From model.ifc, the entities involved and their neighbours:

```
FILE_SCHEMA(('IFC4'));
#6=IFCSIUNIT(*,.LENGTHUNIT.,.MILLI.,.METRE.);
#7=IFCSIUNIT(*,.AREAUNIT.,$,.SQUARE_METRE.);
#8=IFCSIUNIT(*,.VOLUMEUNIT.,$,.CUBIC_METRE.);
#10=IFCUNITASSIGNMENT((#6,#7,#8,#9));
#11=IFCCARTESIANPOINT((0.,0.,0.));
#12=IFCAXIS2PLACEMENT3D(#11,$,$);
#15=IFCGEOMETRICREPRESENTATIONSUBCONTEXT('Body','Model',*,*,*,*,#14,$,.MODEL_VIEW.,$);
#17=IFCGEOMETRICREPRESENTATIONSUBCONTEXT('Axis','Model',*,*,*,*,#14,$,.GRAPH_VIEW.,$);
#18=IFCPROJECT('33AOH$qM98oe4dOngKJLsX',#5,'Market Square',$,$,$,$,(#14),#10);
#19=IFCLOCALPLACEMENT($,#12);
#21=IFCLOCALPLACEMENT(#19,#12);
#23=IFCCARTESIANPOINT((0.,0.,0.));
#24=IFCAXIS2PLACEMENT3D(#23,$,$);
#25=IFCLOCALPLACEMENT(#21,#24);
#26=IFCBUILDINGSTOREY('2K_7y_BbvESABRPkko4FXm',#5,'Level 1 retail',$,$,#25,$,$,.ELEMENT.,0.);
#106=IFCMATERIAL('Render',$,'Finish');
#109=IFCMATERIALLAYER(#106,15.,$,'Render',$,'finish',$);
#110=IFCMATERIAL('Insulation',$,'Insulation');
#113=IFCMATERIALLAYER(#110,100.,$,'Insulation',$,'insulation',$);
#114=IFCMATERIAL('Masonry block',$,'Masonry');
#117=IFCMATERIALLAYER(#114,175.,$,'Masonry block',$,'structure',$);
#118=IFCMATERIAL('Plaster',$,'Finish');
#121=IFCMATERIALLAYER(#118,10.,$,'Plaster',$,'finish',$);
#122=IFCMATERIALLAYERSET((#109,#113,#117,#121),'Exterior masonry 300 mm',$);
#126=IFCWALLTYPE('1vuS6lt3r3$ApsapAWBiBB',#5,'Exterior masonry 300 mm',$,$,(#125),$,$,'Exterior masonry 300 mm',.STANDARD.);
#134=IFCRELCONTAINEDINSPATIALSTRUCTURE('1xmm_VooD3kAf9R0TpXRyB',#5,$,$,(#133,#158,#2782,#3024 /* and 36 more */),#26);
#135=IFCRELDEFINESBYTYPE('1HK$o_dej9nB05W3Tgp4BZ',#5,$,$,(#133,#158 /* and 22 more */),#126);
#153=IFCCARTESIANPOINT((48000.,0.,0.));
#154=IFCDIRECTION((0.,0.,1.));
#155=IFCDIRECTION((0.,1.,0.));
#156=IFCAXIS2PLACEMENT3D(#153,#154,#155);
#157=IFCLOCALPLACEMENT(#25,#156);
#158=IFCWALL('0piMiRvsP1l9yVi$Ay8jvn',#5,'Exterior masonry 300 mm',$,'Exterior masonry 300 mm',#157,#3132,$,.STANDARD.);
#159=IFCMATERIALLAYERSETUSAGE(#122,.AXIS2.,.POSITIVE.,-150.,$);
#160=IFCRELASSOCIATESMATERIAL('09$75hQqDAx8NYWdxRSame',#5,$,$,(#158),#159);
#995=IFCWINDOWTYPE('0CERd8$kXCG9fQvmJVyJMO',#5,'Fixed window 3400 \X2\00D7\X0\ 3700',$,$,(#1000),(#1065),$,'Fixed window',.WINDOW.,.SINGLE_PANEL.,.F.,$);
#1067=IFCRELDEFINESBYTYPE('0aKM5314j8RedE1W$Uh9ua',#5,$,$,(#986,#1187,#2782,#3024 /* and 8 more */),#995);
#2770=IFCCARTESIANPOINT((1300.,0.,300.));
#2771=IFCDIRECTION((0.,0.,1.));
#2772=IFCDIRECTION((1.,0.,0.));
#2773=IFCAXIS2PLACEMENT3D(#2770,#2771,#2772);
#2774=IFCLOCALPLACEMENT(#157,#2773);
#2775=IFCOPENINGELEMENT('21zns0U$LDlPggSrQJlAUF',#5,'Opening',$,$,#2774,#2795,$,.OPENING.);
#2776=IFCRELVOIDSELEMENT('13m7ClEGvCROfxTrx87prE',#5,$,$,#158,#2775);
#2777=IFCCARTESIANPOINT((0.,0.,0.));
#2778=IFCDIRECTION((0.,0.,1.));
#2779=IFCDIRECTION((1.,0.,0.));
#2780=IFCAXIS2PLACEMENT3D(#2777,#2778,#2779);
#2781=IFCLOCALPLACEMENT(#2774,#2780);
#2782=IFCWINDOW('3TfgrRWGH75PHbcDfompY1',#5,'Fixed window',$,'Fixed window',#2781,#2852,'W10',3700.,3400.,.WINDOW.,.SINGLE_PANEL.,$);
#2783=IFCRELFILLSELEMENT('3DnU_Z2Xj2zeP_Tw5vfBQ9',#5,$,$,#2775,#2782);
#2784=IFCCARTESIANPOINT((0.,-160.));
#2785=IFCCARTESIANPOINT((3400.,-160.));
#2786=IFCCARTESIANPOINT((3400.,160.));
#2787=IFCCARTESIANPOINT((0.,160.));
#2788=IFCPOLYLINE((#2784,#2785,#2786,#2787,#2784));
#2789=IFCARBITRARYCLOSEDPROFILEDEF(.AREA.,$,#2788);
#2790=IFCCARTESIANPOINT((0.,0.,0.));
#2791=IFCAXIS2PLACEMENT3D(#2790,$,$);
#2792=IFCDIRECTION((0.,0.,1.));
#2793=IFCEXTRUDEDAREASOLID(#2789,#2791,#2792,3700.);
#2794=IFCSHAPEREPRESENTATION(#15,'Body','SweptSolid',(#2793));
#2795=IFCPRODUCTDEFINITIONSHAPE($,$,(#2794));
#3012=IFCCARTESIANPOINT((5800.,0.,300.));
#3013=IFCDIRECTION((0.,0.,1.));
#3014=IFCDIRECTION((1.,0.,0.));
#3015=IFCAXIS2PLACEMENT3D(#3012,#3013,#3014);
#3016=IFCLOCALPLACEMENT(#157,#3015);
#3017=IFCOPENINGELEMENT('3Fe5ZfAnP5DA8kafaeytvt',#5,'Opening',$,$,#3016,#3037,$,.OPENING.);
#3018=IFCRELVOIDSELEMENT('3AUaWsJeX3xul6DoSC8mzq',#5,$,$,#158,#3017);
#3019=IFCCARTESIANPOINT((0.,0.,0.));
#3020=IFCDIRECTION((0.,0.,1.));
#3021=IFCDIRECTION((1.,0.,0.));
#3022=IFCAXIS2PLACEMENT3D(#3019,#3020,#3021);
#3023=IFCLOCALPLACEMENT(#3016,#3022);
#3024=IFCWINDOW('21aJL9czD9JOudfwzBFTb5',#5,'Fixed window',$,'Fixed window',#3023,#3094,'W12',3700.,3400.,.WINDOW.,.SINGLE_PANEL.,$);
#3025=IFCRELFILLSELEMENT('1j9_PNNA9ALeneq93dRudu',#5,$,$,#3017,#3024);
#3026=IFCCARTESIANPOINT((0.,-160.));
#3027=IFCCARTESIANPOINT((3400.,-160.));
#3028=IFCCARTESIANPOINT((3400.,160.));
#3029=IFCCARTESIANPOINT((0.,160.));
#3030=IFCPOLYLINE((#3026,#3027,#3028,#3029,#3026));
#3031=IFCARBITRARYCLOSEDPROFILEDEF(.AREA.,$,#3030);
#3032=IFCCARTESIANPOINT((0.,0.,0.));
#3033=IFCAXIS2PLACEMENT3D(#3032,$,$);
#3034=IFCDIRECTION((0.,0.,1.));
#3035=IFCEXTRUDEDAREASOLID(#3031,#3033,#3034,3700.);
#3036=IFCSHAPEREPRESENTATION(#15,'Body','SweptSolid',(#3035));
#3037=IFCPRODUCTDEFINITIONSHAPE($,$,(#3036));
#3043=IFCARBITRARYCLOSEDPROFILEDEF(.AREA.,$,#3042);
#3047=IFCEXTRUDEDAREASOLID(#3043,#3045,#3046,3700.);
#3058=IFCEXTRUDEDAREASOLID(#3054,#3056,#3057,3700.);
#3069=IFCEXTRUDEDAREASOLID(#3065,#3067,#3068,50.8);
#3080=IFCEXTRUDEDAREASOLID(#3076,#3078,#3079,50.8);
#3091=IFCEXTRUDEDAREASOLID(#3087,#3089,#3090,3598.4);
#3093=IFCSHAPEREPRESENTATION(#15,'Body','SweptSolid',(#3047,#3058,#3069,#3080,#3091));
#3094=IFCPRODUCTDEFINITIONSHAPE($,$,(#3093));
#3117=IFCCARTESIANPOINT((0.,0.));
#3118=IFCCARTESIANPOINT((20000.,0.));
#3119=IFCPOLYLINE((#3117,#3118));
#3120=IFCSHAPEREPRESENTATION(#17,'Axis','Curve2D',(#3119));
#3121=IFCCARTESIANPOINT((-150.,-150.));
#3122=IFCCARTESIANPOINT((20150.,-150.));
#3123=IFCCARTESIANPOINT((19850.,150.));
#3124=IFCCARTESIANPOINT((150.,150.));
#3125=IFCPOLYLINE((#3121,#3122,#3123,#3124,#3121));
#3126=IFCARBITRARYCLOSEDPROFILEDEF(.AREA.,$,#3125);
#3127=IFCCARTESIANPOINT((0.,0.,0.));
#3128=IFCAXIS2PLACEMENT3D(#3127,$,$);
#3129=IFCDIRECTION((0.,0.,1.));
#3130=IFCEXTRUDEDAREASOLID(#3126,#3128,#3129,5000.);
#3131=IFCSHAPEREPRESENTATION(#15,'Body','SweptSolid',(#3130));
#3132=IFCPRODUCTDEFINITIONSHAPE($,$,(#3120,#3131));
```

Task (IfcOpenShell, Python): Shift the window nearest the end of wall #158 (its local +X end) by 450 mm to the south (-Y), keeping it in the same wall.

```python
import ifcopenshell
import ifcopenshell.api.geometry
import ifcopenshell.util.placement

model = ifcopenshell.open("model.ifc")

window = model.by_guid("21aJL9czD9JOudfwzBFTb5")
opening = window.FillsVoids[0].RelatingOpeningElement
wall = opening.VoidsElements[0].RelatingBuildingElement

wall_matrix = ifcopenshell.util.placement.get_local_placement(wall.ObjectPlacement)
shift = wall_matrix[:3, 0] * -450.0
before = ifcopenshell.util.placement.get_local_placement(window.ObjectPlacement)[:3, 3].copy()

# The window is placed relative to its opening, so it follows when the opening moves.
matrix = ifcopenshell.util.placement.get_local_placement(opening.ObjectPlacement)
matrix[:3, 3] += shift
ifcopenshell.api.geometry.edit_object_placement(
    model, product=opening, matrix=matrix, is_si=False, should_transform_children=True
)

after = ifcopenshell.util.placement.get_local_placement(window.ObjectPlacement)[:3, 3]
print("window moved by", (after - before).round(3) + 0.0)

model.write("model_rev.ifc")
```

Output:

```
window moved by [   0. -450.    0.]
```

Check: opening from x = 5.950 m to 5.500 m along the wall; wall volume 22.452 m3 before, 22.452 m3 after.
